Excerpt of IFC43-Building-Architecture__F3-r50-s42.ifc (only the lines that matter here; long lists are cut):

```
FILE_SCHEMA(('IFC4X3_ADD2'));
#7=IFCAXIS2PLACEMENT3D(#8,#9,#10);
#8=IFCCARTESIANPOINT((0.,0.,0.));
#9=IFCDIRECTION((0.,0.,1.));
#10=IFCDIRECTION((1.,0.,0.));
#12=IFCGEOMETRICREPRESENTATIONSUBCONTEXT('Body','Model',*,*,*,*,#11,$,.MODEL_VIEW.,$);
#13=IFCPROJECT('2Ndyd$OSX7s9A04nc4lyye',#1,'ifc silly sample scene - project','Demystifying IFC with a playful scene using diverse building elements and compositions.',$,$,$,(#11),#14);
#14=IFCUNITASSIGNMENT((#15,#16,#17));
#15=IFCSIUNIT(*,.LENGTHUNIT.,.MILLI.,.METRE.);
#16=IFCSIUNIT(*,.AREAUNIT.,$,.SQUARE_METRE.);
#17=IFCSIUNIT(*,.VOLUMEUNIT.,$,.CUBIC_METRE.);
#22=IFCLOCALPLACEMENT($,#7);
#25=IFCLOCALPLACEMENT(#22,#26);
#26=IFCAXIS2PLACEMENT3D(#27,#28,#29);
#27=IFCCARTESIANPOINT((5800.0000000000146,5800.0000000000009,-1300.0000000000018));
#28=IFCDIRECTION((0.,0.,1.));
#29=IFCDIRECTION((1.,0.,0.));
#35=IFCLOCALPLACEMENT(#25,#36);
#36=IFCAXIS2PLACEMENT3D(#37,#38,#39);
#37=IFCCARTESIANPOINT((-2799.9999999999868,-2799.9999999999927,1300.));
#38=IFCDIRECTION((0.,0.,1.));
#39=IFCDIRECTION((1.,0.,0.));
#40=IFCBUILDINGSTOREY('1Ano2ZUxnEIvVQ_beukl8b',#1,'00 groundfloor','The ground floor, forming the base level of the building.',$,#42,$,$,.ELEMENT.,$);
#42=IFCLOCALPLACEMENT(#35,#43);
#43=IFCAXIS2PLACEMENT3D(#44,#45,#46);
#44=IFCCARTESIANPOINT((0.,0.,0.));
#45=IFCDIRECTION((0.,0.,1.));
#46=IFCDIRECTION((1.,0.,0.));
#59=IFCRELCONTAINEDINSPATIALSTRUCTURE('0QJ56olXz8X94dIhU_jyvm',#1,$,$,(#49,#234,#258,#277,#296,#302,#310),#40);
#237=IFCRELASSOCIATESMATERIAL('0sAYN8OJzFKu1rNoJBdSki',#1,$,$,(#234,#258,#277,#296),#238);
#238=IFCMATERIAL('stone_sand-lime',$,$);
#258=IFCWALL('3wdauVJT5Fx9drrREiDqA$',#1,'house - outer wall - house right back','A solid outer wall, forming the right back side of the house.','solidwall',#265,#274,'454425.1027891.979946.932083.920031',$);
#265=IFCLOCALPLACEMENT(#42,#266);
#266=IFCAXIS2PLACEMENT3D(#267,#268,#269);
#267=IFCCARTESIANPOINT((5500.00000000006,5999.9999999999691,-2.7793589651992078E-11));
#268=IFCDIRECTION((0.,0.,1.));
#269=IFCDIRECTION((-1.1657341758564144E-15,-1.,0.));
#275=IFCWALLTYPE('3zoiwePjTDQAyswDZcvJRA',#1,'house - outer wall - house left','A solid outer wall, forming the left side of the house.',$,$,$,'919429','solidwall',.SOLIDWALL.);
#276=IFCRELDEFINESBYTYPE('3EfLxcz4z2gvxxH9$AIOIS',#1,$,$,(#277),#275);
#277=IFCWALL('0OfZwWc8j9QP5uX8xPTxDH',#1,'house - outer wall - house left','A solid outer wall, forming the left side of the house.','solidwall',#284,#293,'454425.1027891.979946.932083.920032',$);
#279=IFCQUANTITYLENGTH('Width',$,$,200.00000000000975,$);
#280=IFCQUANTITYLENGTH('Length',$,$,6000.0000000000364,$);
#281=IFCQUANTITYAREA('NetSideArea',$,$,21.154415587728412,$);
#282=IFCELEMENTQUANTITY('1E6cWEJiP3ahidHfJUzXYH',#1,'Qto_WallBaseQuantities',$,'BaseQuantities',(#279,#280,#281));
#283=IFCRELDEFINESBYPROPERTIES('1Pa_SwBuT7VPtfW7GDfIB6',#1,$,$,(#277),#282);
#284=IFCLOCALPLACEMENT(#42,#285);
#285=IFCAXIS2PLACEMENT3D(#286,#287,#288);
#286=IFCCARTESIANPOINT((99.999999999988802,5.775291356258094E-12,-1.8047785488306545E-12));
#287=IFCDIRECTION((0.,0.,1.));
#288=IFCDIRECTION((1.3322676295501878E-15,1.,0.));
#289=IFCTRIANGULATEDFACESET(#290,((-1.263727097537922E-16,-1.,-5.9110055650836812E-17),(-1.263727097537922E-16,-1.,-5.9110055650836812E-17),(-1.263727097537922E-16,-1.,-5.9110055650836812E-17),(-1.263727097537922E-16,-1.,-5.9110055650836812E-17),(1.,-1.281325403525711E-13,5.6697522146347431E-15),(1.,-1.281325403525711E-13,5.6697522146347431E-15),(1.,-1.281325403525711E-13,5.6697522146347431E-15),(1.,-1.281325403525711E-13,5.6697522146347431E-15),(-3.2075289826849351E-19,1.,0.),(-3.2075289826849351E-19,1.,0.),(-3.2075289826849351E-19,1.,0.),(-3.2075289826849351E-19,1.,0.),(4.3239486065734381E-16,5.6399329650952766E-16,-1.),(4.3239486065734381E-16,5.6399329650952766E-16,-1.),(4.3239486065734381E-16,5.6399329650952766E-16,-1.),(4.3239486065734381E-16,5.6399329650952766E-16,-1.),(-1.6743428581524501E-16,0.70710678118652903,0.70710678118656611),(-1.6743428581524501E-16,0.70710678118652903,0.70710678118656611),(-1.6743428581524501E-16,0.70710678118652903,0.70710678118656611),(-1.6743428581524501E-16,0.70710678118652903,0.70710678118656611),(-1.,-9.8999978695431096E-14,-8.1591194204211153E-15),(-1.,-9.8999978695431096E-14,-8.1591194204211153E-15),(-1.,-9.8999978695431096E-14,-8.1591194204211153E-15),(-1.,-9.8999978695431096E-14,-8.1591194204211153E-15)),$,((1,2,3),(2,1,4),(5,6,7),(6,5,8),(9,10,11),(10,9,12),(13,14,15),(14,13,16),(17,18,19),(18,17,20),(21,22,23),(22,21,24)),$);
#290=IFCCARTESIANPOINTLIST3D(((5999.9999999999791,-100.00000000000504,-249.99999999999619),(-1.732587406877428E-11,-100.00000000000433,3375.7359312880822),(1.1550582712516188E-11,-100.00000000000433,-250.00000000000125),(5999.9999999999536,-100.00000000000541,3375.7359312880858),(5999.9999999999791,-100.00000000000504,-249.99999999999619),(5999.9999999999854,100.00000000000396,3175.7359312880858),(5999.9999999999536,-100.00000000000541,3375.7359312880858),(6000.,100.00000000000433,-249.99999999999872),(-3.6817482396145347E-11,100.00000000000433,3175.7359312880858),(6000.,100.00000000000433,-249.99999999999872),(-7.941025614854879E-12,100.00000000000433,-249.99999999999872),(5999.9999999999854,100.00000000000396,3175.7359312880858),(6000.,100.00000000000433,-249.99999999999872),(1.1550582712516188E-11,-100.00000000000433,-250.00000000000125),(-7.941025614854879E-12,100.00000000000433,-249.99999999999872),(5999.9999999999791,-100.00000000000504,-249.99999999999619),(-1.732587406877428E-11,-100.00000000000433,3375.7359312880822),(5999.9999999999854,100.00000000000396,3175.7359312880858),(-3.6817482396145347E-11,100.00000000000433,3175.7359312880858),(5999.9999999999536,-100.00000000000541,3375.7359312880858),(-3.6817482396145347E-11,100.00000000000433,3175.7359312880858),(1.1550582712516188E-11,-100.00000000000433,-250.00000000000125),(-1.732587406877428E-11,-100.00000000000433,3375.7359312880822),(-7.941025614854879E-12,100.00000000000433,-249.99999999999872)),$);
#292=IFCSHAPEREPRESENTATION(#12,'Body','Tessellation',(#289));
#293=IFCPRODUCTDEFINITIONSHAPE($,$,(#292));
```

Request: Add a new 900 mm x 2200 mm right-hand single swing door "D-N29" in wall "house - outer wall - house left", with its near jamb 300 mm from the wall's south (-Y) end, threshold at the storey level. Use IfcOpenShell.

```python
import numpy as np
import ifcopenshell
import ifcopenshell.api.feature
import ifcopenshell.api.geometry
import ifcopenshell.api.pset
import ifcopenshell.api.root
import ifcopenshell.api.spatial
import ifcopenshell.geom
import ifcopenshell.util.element
import ifcopenshell.util.placement
import ifcopenshell.util.representation
import ifcopenshell.util.shape
import ifcopenshell.util.unit

model = ifcopenshell.open("IFC43-Building-Architecture__F3-r50-s42.ifc")
unit_scale = ifcopenshell.util.unit.calculate_unit_scale(model)
area_scale = ifcopenshell.util.unit.calculate_unit_scale(model, "AREAUNIT")
settings = ifcopenshell.geom.settings()


def volume(element):
    """Net volume in cubic metres, openings subtracted."""
    shape = ifcopenshell.geom.create_shape(settings, element)
    return ifcopenshell.util.shape.get_volume(shape.geometry)


wall = model.by_guid("0OfZwWc8j9QP5uX8xPTxDH")
storey = ifcopenshell.util.element.get_container(wall, ifc_class="IfcBuildingStorey")
context = ifcopenshell.util.representation.get_context(model, "Model", "Body", "MODEL_VIEW")
before = volume(wall)

width, height, from_end, sill = 0.9, 2.2, 0.3, 0.0  # metres

# The wall runs along its own X axis, and the end named is its -X end.
wall_shape = ifcopenshell.geom.create_shape(settings, wall)
x, y, z = ifcopenshell.util.shape.get_vertices(wall_shape.geometry).T
start = x.min() + from_end
face, thickness = float(y.min()), float(y.max() - y.min())
wall_matrix = ifcopenshell.util.placement.get_local_placement(wall.ObjectPlacement)
level = ifcopenshell.util.placement.get_local_placement(storey.ObjectPlacement)[2, 3]


def in_wall(x, y):
    """Placement at x, y metres in the wall's axes, at sill height."""
    matrix = wall_matrix.copy()
    matrix[:, 3] = wall_matrix @ np.array([x / unit_scale, y / unit_scale, 0.0, 1.0])
    matrix[2, 3] = level + sill / unit_scale
    return matrix


# Opening: a box that overshoots both wall faces by 50 mm.
opening = ifcopenshell.api.root.create_entity(model, ifc_class="IfcOpeningElement", predefined_type="OPENING")
box = ifcopenshell.api.geometry.add_wall_representation(
    model, context=context, length=width, height=height, thickness=thickness + 0.1
)
ifcopenshell.api.geometry.assign_representation(model, product=opening, representation=box)
ifcopenshell.api.geometry.edit_object_placement(model, product=opening, matrix=in_wall(start, face - 0.05), is_si=False)
ifcopenshell.api.feature.add_feature(model, feature=opening, element=wall)

door = ifcopenshell.api.root.create_entity(model, ifc_class="IfcDoor", name="D-N29", predefined_type="DOOR")
door.OverallWidth, door.OverallHeight = width / unit_scale, height / unit_scale
door.OperationType = "SINGLE_SWING_RIGHT"
body = ifcopenshell.api.geometry.add_door_representation(
    model,
    context=context,
    overall_width=door.OverallWidth,
    overall_height=door.OverallHeight,
    operation_type="SINGLE_SWING_RIGHT",
    lining_properties={"LiningDepth": thickness / unit_scale, "ThresholdDepth": thickness / unit_scale},
)
ifcopenshell.api.geometry.assign_representation(model, product=door, representation=body)
ifcopenshell.api.spatial.assign_container(model, products=[door], relating_structure=storey)
ifcopenshell.api.feature.add_filling(model, opening=opening, element=door)

# The lining spans the wall, so the door starts at the wall face.
ifcopenshell.api.geometry.edit_object_placement(model, product=door, matrix=in_wall(start, face), is_si=False)

after = volume(wall)

# Update the wall's stored quantities.
qto = model.by_id(ifcopenshell.util.element.get_pset(wall, "Qto_WallBaseQuantities", should_inherit=False)["id"])
ifcopenshell.api.pset.edit_qto(model, qto=qto, properties={"NetSideArea": after / thickness / area_scale})

print(f"wall volume {before:.3f} -> {after:.3f} m3")

model.write("IFC43-Building-Architecture__F3-r50-s42_updated.ifc")
```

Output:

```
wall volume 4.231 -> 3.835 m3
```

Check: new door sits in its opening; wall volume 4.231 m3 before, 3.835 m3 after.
